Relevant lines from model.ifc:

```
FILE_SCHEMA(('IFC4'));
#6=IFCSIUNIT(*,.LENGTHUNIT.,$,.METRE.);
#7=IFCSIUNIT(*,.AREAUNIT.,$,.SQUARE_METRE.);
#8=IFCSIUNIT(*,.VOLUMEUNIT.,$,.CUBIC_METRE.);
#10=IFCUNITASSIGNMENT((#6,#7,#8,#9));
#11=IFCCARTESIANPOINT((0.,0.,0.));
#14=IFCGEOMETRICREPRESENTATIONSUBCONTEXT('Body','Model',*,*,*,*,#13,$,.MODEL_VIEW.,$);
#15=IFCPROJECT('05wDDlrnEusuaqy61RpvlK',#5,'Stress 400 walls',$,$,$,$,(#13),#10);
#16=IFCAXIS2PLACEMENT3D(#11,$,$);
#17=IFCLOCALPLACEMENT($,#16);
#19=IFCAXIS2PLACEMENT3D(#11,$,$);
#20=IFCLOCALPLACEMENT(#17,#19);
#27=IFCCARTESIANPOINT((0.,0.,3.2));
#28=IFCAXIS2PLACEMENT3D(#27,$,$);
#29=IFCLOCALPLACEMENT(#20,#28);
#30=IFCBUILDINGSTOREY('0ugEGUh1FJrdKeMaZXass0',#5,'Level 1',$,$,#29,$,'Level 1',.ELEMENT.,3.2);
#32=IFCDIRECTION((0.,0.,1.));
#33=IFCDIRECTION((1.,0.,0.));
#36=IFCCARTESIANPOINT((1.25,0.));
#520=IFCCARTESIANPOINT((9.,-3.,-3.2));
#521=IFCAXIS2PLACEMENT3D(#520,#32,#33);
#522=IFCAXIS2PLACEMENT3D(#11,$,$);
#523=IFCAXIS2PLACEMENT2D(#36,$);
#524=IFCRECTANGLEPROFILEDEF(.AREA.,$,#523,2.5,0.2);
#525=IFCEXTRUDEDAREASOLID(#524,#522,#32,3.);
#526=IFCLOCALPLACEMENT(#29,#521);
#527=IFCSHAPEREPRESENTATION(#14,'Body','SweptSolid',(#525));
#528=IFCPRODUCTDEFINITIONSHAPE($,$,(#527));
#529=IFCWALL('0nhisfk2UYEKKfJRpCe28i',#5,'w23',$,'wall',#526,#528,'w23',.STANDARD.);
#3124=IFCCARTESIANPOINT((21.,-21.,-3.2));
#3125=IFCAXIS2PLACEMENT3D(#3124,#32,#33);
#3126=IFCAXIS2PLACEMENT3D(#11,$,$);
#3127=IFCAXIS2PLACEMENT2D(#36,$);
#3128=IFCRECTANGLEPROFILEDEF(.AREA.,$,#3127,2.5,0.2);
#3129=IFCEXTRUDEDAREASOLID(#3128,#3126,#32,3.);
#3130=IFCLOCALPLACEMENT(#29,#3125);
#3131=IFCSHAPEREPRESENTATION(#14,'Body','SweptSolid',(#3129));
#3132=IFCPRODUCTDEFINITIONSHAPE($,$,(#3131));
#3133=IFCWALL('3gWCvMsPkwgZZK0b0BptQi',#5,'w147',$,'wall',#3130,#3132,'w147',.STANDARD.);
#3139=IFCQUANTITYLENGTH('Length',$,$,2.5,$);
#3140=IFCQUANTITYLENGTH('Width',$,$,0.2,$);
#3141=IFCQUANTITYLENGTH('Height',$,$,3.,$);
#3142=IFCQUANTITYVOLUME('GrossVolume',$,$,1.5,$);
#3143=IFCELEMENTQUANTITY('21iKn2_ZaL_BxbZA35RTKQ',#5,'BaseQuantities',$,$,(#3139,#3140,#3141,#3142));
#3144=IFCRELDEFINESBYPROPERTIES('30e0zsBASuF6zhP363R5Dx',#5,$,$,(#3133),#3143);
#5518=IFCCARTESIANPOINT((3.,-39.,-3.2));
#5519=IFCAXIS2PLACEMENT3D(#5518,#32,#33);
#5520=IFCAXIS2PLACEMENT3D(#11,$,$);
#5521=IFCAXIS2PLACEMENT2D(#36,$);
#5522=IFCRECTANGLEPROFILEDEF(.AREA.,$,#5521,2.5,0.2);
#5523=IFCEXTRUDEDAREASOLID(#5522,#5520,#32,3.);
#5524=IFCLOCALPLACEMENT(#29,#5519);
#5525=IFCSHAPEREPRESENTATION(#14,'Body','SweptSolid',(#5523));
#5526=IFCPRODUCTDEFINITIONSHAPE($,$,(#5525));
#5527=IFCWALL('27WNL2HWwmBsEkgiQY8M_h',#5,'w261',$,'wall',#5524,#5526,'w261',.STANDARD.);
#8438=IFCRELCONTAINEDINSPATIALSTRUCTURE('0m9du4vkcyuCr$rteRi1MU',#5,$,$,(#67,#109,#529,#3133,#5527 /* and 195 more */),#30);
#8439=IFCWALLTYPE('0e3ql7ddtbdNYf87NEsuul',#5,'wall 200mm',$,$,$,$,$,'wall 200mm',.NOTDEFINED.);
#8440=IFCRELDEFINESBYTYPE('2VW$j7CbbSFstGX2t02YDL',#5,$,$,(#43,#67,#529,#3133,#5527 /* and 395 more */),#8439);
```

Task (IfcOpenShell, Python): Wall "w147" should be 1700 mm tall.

```python
import ifcopenshell
import ifcopenshell.api.pset
import ifcopenshell.geom
import ifcopenshell.util.element
import ifcopenshell.util.representation
import ifcopenshell.util.shape
import ifcopenshell.util.unit

model = ifcopenshell.open("model.ifc")
unit_scale = ifcopenshell.util.unit.calculate_unit_scale(model)
volume_scale = ifcopenshell.util.unit.calculate_unit_scale(model, "VOLUMEUNIT")
settings = ifcopenshell.geom.settings()


def volume(element):
    """Net volume in cubic metres, openings subtracted."""
    shape = ifcopenshell.geom.create_shape(settings, element)
    return ifcopenshell.util.shape.get_volume(shape.geometry)


wall = model.by_id(3133)
before = volume(wall)

body = ifcopenshell.util.representation.get_representation(wall, "Model", "Body")
solid = body.Items[0]
old_height = solid.Depth
solid.Depth = 1.7 / unit_scale
after = volume(wall)

# Update the stored height, areas and volumes.
qto = model.by_id(ifcopenshell.util.element.get_pset(wall, "BaseQuantities", should_inherit=False)["id"])
ifcopenshell.api.pset.edit_qto(model, qto=qto, properties={
    "Height": solid.Depth,
    "GrossVolume": ifcopenshell.util.element.get_pset(wall, "BaseQuantities", "GrossVolume") * solid.Depth / old_height,
})

print(f"height {old_height:g} -> {solid.Depth:g}, volume {before:.3f} -> {after:.3f} m3")

model.write("model_edited.ifc")
```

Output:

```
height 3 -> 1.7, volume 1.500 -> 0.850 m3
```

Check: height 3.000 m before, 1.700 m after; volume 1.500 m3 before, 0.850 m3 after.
